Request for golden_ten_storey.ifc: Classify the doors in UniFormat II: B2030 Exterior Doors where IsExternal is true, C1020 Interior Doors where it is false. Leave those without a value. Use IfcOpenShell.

First a look at what the model holds.

```python
import ifcopenshell
import ifcopenshell.util.element

model = ifcopenshell.open("golden_ten_storey.ifc")
print(model.schema)
print("classifications:", [c.Name for c in model.by_type("IfcClassification")])
values = [ifcopenshell.util.element.get_pset(e, "Pset_DoorCommon", "IsExternal") for e in model.by_type("IfcDoor")]
for value in (True, False, None):
    print("IsExternal", value, values.count(value))
```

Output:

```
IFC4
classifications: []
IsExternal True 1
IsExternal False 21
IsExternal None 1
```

```python
import ifcopenshell
import ifcopenshell.api.classification
import ifcopenshell.util.element

model = ifcopenshell.open("golden_ten_storey.ifc")

system = ifcopenshell.api.classification.add_classification(model, classification="UniFormat II")

doors = model.by_type("IfcDoor")
external = {e: ifcopenshell.util.element.get_pset(e, "Pset_DoorCommon", "IsExternal") for e in doors}
for flag, code, name in ((True, "B2030", "Exterior Doors"), (False, "C1020", "Interior Doors")):
    products = [e for e in doors if external[e] is flag]
    ifcopenshell.api.classification.add_reference(
        model, products=products, classification=system, identification=code, name=name
    )
    print(code, len(products))

model.write("golden_ten_storey_rev.ifc")
```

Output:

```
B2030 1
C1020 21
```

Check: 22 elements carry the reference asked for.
